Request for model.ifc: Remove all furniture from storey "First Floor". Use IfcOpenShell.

First a look at what the model holds.

```python
import ifcopenshell
import ifcopenshell.util.element

model = ifcopenshell.open("model.ifc")
print(model.schema)
storey = next(s for s in model.by_type("IfcBuildingStorey") if s.Name == "First Floor")
furniture = [e for e in ifcopenshell.util.element.get_decomposition(storey) if e.is_a("IfcFurnishingElement")]
seen = {}
for e in furniture:
    element_type = ifcopenshell.util.element.get_type(e)
    name = element_type.Name if element_type not in (None, e) else None
    seen[name] = seen.get(name, 0) + 1
for name, count in sorted(seen.items(), key=str):
    print(count, "x", name)
```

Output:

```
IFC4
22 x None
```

```python
import ifcopenshell
import ifcopenshell.api.root
import ifcopenshell.util.element

model = ifcopenshell.open("model.ifc")

storey = next(s for s in model.by_type("IfcBuildingStorey") if s.Name == "First Floor")
furniture = [e for e in ifcopenshell.util.element.get_decomposition(storey) if e.is_a("IfcFurnishingElement")]

for e in furniture:
    ifcopenshell.api.root.remove_product(model, product=e)
print(len(furniture), "removed")

model.write("model-out.ifc")
```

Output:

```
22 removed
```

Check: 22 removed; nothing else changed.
